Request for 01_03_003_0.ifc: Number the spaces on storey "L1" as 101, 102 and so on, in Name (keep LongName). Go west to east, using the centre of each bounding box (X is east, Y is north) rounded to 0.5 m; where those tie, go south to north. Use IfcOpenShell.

First a look at what the model holds.

```python
import ifcopenshell
import ifcopenshell.util.element
import ifcopenshell.util.placement

model = ifcopenshell.open("01_03_003_0.ifc")
print(model.schema)
storey = next(s for s in model.by_type("IfcBuildingStorey") if s.Name == "L1")
spaces = [e for e in ifcopenshell.util.element.get_decomposition(storey) if e.is_a("IfcSpace")]
for e in sorted(spaces, key=lambda e: e.id()):
    origin = ifcopenshell.util.placement.get_local_placement(e.ObjectPlacement)[:3, 3]
    print(e.id(), e.Name, e.LongName, origin.round(2) + 0.0, sep=" | ")
```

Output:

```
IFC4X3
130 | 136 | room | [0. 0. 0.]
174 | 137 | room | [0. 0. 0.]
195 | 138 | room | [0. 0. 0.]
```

```python
import ifcopenshell
import ifcopenshell.geom
import ifcopenshell.util.element
import ifcopenshell.util.shape

model = ifcopenshell.open("01_03_003_0.ifc")
settings = ifcopenshell.geom.settings()
settings.set("use-world-coords", True)


def centre(element):
    shape = ifcopenshell.geom.create_shape(settings, element)
    return ifcopenshell.util.shape.get_bbox_centroid(shape.geometry)


storey = next(s for s in model.by_type("IfcBuildingStorey") if s.Name == "L1")
spaces = [e for e in ifcopenshell.util.element.get_decomposition(storey) if e.is_a("IfcSpace")]

# Insertion points can sit at a corner or the storey origin, so sort by the geometry (in metres).
centres = {e: centre(e) for e in spaces}
spaces.sort(key=lambda e: (round(centres[e][0] / 0.5), centres[e][1]))

for i, e in enumerate(spaces, start=1):
    number = f"1{i:02d}"
    e.Name = number
    print(e.id(), number)

model.write("01_03_003_0-out.ifc")
```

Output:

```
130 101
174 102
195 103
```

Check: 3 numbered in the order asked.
